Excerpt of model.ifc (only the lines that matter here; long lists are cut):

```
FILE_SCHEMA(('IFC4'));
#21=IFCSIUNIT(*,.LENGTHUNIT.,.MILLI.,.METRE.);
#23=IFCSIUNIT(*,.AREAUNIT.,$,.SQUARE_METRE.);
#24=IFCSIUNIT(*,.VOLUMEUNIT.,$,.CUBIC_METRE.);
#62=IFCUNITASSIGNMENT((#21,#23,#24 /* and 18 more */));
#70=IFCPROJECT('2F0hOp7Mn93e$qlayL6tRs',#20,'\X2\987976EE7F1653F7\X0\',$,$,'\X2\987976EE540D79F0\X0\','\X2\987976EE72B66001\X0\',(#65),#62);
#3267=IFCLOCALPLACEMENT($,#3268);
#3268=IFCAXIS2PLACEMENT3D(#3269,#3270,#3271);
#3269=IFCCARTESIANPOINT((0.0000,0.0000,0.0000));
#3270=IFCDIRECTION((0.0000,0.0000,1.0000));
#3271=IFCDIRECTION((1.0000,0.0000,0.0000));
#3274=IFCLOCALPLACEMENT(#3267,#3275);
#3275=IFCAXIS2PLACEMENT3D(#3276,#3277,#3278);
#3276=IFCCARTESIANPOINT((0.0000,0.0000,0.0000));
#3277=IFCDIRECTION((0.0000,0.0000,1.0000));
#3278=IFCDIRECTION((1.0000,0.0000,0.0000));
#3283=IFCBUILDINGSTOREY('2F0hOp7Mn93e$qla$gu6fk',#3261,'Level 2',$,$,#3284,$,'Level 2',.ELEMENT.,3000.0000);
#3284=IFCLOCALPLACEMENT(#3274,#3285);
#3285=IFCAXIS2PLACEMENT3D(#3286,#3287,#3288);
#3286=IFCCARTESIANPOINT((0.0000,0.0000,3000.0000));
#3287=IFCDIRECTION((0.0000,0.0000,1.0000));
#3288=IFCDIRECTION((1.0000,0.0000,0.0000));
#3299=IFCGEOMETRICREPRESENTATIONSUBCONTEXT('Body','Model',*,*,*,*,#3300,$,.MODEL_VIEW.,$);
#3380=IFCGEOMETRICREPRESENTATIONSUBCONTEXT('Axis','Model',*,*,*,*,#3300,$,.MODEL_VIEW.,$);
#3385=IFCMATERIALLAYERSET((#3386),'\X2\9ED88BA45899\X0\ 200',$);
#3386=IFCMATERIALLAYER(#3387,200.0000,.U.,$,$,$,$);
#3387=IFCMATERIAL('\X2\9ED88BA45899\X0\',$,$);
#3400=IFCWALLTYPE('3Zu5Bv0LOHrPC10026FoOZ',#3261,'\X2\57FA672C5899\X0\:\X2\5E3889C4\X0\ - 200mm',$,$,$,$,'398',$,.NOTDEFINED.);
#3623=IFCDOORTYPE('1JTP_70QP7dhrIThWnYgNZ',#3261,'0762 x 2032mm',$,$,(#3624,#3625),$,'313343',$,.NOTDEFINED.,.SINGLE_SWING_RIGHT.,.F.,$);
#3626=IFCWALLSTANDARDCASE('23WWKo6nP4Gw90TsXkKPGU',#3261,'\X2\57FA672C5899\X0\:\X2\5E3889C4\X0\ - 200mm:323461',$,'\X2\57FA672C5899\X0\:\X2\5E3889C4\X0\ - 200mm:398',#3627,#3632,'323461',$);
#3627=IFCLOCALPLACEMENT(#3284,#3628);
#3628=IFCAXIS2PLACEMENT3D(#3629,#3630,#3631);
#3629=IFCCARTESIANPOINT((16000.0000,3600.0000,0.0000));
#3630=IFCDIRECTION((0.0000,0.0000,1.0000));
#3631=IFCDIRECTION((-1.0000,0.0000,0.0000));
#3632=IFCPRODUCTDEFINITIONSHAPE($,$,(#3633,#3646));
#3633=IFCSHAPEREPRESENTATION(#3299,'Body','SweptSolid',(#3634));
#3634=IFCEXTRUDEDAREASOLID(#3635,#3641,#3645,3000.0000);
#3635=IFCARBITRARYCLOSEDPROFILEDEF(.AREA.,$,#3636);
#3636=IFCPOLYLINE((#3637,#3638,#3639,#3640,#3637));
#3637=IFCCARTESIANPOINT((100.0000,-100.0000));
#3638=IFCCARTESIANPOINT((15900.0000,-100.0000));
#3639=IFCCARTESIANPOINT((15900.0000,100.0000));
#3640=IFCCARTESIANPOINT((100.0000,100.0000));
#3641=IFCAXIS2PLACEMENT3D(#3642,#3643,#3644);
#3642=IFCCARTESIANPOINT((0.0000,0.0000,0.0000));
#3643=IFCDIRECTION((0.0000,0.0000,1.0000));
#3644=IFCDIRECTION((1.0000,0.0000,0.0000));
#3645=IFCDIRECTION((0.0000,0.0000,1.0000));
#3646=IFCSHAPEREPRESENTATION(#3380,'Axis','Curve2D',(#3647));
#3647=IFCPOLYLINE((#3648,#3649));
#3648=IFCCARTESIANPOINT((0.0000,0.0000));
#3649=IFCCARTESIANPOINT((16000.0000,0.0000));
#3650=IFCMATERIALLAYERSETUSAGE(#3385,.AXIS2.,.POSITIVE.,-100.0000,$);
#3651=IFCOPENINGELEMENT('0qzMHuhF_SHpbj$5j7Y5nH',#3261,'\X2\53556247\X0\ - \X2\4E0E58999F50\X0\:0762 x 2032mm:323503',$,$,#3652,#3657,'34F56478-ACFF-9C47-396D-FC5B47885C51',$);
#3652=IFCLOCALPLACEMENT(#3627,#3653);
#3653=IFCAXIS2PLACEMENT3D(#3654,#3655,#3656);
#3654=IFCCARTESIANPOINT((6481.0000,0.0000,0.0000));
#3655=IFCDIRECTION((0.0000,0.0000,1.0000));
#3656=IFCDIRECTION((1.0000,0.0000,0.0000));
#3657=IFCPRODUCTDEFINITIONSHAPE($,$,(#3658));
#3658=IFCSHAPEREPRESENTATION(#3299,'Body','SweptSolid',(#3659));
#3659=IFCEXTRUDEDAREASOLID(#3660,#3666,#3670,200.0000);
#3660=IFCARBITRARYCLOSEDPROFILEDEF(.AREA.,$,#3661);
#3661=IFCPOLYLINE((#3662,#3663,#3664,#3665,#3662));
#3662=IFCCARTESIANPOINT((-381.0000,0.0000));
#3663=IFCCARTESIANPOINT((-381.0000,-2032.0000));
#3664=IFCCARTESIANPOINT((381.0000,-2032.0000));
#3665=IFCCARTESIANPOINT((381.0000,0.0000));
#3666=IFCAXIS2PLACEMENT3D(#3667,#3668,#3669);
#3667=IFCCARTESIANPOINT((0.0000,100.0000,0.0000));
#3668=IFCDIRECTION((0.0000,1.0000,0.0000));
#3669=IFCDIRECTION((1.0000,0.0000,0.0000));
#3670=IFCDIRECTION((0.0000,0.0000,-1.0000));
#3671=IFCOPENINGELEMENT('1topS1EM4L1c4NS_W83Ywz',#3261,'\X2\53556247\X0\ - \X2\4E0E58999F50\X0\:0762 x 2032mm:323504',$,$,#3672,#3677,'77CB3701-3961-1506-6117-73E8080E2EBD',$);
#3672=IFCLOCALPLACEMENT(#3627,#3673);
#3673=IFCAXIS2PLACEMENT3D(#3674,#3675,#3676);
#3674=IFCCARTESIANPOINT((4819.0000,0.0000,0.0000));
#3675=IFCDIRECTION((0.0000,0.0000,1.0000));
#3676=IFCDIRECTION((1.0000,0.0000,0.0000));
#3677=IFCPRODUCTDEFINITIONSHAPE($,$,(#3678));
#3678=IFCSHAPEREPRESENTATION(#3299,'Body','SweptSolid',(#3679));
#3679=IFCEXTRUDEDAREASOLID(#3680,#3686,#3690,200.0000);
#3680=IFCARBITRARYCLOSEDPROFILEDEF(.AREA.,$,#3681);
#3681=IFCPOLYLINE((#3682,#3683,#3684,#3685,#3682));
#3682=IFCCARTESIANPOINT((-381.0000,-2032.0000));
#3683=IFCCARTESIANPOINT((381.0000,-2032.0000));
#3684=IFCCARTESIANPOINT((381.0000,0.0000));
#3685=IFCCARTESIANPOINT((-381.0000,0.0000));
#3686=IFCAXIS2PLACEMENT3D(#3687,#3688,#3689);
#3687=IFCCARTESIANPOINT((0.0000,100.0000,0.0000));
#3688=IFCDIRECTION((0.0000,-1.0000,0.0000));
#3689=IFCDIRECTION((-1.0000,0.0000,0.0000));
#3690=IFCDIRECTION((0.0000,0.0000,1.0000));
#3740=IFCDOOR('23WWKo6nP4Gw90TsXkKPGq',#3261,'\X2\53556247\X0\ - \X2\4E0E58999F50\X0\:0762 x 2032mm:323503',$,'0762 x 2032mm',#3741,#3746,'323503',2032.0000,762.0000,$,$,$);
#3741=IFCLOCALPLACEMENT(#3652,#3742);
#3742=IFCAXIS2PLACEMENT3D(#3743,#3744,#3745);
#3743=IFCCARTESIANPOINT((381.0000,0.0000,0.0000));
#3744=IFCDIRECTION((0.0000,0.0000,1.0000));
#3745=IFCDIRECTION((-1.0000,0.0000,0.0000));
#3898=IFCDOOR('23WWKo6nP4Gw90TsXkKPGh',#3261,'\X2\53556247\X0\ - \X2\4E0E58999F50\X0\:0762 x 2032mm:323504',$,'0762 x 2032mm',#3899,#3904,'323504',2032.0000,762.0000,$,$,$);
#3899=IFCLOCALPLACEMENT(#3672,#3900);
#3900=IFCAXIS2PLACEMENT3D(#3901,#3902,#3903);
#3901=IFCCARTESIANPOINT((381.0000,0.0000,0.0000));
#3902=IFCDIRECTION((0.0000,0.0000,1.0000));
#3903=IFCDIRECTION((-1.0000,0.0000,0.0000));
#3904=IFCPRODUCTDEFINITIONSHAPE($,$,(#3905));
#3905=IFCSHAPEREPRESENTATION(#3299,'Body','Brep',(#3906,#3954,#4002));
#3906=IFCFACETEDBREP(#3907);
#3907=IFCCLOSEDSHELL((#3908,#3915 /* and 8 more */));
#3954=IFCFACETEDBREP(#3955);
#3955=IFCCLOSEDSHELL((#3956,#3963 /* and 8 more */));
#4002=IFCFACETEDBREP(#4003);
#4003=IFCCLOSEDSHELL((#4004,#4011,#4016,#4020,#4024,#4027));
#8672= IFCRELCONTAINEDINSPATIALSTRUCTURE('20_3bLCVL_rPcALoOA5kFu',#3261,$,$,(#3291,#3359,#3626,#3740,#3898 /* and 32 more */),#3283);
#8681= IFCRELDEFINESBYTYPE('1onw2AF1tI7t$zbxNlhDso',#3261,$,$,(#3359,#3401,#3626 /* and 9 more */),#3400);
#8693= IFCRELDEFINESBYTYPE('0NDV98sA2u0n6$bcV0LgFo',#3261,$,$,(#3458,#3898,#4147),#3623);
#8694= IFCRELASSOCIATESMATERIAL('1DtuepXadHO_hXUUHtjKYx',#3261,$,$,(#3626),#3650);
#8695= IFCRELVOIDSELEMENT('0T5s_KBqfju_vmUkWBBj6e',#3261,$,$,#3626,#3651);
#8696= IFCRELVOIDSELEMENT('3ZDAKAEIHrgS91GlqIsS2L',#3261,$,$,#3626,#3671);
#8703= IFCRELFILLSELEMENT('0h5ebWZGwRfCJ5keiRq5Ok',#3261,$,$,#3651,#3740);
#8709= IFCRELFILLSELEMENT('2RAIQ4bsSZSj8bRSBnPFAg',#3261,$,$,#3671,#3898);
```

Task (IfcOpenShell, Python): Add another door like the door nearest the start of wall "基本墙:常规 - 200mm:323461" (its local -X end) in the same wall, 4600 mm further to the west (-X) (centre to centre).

```python
import ifcopenshell
import ifcopenshell.api.feature
import ifcopenshell.api.geometry
import ifcopenshell.api.root
import ifcopenshell.geom
import ifcopenshell.util.element
import ifcopenshell.util.placement
import ifcopenshell.util.shape
import ifcopenshell.util.unit

model = ifcopenshell.open("model.ifc")
unit_scale = ifcopenshell.util.unit.calculate_unit_scale(model)
settings = ifcopenshell.geom.settings()


def volume(element):
    """Net volume in cubic metres, openings subtracted."""
    shape = ifcopenshell.geom.create_shape(settings, element)
    return ifcopenshell.util.shape.get_volume(shape.geometry)


def reuse_history(source, copy):
    """copy_class also copies each property set's owner history, people and application; keep the originals."""
    for rel in copy.IsDefinedBy:
        if rel.is_a("IfcRelDefinesByProperties") and (history := rel.RelatingPropertyDefinition.OwnerHistory):
            rel.RelatingPropertyDefinition.OwnerHistory = source.OwnerHistory
            ifcopenshell.util.element.remove_deep2(model, history)


door = model.by_guid("23WWKo6nP4Gw90TsXkKPGh")
opening = door.FillsVoids[0].RelatingOpeningElement
wall = opening.VoidsElements[0].RelatingBuildingElement
before = volume(wall)
shift = ifcopenshell.util.placement.get_local_placement(wall.ObjectPlacement)[:3, 0] * 4.6 / unit_scale

# copy_class copies the void relationship, type, container and properties, but no geometry.
new_opening = ifcopenshell.api.root.copy_class(model, product=opening)
new_opening.Representation = ifcopenshell.util.element.copy_deep(
    model, opening.Representation, exclude=["IfcGeometricRepresentationContext", "IfcRepresentationMap"]
)
new_opening.Name = "单扇 - 与墙齐:0762 x 2032mm"
new_opening.Tag = None
new_door = ifcopenshell.api.root.copy_class(model, product=door)
new_door.Representation = ifcopenshell.util.element.copy_deep(
    model, door.Representation, exclude=["IfcGeometricRepresentationContext", "IfcRepresentationMap"]
)
new_door.Name = "单扇 - 与墙齐:0762 x 2032mm"
new_door.Tag = None
reuse_history(door, new_door)
ifcopenshell.api.feature.add_filling(model, opening=new_opening, element=new_door)

for old, new in ((opening, new_opening), (door, new_door)):
    matrix = ifcopenshell.util.placement.get_local_placement(old.ObjectPlacement)
    matrix[:3, 3] += shift
    ifcopenshell.api.geometry.edit_object_placement(model, product=new, matrix=matrix, is_si=False)

after = volume(wall)

print(f"wall volume {before:.3f} -> {after:.3f} m3")

model.write("model_v2.ifc")
```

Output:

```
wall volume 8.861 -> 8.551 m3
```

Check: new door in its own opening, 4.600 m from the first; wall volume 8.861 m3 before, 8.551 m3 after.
